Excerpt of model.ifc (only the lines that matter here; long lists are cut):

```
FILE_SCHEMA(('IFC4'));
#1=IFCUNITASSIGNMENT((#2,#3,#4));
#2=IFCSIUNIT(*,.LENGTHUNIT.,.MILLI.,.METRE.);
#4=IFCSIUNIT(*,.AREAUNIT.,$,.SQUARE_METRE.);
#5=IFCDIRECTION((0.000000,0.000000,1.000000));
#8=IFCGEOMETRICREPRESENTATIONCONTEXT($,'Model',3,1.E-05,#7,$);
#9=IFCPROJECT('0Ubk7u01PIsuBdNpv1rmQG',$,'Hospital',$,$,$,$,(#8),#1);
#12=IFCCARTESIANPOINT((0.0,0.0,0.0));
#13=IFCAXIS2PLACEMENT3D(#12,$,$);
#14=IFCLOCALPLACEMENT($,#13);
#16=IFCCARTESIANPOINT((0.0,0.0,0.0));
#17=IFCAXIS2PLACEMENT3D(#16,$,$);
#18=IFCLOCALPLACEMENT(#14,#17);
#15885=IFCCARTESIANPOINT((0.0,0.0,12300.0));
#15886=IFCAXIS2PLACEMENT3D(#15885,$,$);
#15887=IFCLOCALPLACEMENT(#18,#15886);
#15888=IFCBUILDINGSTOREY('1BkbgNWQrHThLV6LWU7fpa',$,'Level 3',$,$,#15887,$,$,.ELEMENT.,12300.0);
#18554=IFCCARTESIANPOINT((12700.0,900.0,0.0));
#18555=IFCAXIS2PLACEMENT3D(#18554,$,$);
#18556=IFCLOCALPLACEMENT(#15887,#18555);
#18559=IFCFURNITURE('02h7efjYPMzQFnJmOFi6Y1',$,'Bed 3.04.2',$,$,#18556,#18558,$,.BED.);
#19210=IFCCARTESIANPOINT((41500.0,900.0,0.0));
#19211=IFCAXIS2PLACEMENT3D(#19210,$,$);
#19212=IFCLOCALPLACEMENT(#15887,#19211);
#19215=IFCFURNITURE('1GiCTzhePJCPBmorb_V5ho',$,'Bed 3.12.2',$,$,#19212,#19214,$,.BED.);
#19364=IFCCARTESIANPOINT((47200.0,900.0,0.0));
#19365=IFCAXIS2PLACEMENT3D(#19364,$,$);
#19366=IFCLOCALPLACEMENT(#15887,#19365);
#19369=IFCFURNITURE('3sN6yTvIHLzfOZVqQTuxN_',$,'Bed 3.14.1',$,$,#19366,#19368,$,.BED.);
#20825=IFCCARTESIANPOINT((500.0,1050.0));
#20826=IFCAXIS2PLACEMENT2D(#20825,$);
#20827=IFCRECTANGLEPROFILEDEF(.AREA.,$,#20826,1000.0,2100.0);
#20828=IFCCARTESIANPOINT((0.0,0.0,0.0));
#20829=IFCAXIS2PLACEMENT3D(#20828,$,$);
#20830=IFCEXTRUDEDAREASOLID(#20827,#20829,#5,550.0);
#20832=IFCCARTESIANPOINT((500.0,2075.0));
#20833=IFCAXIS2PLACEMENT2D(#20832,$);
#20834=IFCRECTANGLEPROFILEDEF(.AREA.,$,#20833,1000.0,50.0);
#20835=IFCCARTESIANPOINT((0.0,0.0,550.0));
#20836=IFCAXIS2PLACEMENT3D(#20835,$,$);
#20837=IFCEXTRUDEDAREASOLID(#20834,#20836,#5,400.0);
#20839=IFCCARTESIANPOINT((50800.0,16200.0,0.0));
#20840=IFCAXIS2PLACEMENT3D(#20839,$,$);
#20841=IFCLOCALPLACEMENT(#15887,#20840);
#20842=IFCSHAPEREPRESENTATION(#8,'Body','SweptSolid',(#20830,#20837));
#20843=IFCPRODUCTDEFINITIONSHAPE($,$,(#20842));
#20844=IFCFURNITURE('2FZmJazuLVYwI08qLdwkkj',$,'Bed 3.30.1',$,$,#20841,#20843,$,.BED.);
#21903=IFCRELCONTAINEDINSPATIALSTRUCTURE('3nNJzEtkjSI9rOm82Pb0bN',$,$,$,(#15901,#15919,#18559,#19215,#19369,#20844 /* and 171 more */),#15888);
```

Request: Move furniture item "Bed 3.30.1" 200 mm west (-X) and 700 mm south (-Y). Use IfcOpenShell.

```python
import ifcopenshell
import ifcopenshell.api.geometry
import ifcopenshell.util.placement
import ifcopenshell.util.unit

model = ifcopenshell.open("model.ifc")
unit_scale = ifcopenshell.util.unit.calculate_unit_scale(model)

item = model.by_guid("2FZmJazuLVYwI08qLdwkkj")
matrix = ifcopenshell.util.placement.get_local_placement(item.ObjectPlacement)
matrix[0, 3] -= 0.2 / unit_scale
matrix[1, 3] -= 0.7 / unit_scale
ifcopenshell.api.geometry.edit_object_placement(model, product=item, matrix=matrix, is_si=False)

print(ifcopenshell.util.placement.get_local_placement(item.ObjectPlacement).round(3) + 0.0)

model.write("model_v2.ifc")
```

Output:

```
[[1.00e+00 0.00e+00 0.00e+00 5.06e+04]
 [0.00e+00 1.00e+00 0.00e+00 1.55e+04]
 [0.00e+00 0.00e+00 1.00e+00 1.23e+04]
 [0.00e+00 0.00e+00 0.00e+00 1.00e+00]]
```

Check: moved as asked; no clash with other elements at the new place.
